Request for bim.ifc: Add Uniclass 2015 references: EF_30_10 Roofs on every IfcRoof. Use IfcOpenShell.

First a look at what the model holds.

```python
import ifcopenshell

model = ifcopenshell.open("bim.ifc")
print(model.schema)
print("classifications:", [c.Name for c in model.by_type("IfcClassification")])
for ifc_class in ("IfcDoor", "IfcRoof", "IfcStair", "IfcWall", "IfcWindow"):
    print(ifc_class, len(model.by_type(ifc_class)))
```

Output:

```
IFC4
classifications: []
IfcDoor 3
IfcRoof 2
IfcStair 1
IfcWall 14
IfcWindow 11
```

```python
import ifcopenshell
import ifcopenshell.api.classification

model = ifcopenshell.open("bim.ifc")

system = ifcopenshell.api.classification.add_classification(model, classification="Uniclass 2015")

codes = {
    "IfcRoof": ("EF_30_10", "Roofs"),
}
for ifc_class, (code, name) in codes.items():
    products = model.by_type(ifc_class)
    ifcopenshell.api.classification.add_reference(
        model, products=products, classification=system, identification=code, name=name
    )
    print(code, len(products))

model.write("bim-out.ifc")
```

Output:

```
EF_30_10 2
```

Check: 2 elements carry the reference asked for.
